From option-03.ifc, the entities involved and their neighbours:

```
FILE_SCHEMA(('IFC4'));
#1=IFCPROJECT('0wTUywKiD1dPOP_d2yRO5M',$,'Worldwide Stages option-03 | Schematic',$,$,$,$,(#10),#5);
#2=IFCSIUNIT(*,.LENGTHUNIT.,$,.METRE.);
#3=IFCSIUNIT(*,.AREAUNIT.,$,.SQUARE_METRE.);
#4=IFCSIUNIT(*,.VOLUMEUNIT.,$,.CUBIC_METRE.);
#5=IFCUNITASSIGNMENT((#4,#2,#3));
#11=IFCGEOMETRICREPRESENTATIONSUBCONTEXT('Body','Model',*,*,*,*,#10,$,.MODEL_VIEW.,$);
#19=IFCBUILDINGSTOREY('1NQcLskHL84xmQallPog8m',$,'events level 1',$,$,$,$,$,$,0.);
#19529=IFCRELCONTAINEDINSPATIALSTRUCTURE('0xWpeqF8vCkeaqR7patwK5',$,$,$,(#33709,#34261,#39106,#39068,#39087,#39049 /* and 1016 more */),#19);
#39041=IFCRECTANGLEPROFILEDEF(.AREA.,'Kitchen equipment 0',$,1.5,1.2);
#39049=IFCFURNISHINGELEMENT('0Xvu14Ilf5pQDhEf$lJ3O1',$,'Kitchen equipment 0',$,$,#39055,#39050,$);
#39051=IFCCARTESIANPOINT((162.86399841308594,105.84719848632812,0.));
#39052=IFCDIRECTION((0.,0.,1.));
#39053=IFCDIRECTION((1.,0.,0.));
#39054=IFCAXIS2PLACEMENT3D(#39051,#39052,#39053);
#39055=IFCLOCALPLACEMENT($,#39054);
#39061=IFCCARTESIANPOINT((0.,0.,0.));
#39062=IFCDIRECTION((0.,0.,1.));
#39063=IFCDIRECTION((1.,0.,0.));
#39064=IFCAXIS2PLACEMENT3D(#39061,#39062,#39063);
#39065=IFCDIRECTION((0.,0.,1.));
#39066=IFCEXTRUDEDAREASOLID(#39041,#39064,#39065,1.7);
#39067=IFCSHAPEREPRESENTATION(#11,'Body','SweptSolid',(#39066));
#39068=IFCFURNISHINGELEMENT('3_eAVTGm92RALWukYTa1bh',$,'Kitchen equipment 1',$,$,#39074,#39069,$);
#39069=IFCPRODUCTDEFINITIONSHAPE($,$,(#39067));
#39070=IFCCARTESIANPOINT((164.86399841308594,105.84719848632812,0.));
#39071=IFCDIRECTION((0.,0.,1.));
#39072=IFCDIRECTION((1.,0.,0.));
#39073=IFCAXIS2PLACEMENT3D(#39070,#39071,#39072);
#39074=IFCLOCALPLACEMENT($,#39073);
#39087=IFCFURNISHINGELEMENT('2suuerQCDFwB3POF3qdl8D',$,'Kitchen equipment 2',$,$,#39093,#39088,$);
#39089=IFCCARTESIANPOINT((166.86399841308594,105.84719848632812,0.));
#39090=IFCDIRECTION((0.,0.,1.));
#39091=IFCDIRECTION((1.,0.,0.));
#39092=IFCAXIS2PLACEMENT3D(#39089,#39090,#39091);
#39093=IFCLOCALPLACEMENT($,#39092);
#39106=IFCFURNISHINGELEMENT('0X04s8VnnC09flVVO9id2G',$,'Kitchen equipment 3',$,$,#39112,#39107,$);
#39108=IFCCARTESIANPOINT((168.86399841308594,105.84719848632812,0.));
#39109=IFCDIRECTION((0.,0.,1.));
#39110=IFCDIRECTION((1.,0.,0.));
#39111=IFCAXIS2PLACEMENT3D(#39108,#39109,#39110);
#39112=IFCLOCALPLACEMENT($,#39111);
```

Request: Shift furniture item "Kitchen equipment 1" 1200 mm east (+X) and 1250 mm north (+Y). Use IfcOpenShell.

```python
import ifcopenshell
import ifcopenshell.api.geometry
import ifcopenshell.util.placement
import ifcopenshell.util.unit

model = ifcopenshell.open("option-03.ifc")
unit_scale = ifcopenshell.util.unit.calculate_unit_scale(model)

item = model.by_guid("3_eAVTGm92RALWukYTa1bh")
matrix = ifcopenshell.util.placement.get_local_placement(item.ObjectPlacement)
matrix[0, 3] += 1.2 / unit_scale
matrix[1, 3] += 1.25 / unit_scale
ifcopenshell.api.geometry.edit_object_placement(model, product=item, matrix=matrix, is_si=False)

print(ifcopenshell.util.placement.get_local_placement(item.ObjectPlacement).round(3) + 0.0)

model.write("option-03_edited.ifc")
```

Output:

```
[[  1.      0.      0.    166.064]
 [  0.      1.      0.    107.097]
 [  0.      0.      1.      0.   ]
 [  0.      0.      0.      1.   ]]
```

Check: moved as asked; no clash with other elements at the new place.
